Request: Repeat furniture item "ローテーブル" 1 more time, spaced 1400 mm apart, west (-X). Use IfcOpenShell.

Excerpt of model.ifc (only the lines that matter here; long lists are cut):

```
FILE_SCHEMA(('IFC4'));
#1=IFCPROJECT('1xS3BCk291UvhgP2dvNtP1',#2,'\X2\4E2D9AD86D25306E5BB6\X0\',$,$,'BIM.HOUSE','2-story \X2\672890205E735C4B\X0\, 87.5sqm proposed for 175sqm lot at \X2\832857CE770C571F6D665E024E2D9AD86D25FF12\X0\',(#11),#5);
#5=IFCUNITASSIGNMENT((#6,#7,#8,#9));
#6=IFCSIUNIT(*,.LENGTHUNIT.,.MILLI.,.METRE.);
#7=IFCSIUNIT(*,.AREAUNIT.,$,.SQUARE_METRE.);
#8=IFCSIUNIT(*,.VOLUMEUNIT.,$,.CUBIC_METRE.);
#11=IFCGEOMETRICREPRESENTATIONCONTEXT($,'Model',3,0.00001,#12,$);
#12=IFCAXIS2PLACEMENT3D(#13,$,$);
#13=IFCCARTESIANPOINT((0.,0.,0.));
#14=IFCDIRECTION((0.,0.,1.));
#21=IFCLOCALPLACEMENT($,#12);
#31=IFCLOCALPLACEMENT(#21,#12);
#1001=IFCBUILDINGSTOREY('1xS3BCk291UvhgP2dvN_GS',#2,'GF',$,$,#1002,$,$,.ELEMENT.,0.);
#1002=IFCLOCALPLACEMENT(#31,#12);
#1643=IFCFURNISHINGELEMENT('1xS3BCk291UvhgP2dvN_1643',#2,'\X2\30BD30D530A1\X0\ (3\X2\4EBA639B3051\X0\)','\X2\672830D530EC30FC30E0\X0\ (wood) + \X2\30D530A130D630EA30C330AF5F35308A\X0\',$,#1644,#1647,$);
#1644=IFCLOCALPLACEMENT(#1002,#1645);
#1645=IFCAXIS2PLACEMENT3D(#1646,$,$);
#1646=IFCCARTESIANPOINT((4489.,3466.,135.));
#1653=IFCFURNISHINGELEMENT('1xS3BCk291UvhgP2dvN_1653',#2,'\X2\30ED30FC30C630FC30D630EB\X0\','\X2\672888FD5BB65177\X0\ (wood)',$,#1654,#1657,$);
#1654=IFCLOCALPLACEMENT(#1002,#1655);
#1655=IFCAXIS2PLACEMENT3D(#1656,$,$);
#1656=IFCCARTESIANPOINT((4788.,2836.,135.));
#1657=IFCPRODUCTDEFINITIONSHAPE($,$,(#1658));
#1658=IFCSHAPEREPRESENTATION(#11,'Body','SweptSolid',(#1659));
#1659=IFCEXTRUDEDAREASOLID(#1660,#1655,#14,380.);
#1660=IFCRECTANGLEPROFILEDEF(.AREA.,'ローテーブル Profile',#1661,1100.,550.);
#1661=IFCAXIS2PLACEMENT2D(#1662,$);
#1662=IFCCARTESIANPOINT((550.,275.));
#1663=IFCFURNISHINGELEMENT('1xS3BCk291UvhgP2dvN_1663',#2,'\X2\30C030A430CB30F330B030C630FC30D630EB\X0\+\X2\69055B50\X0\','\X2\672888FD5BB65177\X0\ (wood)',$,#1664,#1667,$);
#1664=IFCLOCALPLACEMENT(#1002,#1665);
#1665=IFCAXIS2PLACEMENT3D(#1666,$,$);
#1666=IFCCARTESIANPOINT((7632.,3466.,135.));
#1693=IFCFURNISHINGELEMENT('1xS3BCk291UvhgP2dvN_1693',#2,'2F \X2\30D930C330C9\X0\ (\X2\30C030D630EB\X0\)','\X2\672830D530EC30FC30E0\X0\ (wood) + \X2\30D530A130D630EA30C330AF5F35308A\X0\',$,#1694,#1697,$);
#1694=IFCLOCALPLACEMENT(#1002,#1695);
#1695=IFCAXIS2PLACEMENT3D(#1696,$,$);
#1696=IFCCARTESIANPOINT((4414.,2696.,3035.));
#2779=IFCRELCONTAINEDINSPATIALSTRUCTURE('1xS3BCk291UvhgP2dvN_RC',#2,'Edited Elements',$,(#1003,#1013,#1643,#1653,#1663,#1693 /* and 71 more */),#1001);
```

```python
import numpy as np
import ifcopenshell
import ifcopenshell.api.geometry
import ifcopenshell.api.root
import ifcopenshell.util.element
import ifcopenshell.util.placement
import ifcopenshell.util.unit

model = ifcopenshell.open("model.ifc")
unit_scale = ifcopenshell.util.unit.calculate_unit_scale(model)


def reuse_history(source, copy):
    """copy_class also copies each property set's owner history, people and application; keep the originals."""
    for rel in copy.IsDefinedBy:
        if rel.is_a("IfcRelDefinesByProperties") and (history := rel.RelatingPropertyDefinition.OwnerHistory):
            rel.RelatingPropertyDefinition.OwnerHistory = source.OwnerHistory
            ifcopenshell.util.element.remove_deep2(model, history)


source = model.by_guid("1xS3BCk291UvhgP2dvN_1653")
base = ifcopenshell.util.placement.get_local_placement(source.ObjectPlacement)
step = np.array([-1.0, 0.0, 0.0]) * 1.4 / unit_scale

for i in range(1, 2):
    copy = ifcopenshell.api.root.copy_class(model, product=source)
    copy.Representation = ifcopenshell.util.element.copy_deep(
        model, source.Representation, exclude=["IfcGeometricRepresentationContext", "IfcRepresentationMap"]
    )
    reuse_history(source, copy)
    matrix = base.copy()
    matrix[:3, 3] += i * step
    print("added at", matrix[:3, 3].round(3) + 0.0)
    ifcopenshell.api.geometry.edit_object_placement(model, product=copy, matrix=matrix, is_si=False)

model.write("model_rev.ifc")
```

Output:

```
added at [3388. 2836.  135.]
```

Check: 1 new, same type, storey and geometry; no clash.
